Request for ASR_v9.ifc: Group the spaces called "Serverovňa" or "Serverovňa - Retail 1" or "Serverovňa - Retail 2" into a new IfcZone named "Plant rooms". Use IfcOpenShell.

First a look at what the model holds.

```python
import ifcopenshell

model = ifcopenshell.open("ASR_v9.ifc")
print(model.schema)
seen = {}
for space in model.by_type("IfcSpace"):
    seen[space.LongName] = seen.get(space.LongName, 0) + 1
for name, count in sorted(seen.items(), key=str):
    print(count, "x", name)
print("zones:", [z.Name for z in model.by_type("IfcZone")][:20])
```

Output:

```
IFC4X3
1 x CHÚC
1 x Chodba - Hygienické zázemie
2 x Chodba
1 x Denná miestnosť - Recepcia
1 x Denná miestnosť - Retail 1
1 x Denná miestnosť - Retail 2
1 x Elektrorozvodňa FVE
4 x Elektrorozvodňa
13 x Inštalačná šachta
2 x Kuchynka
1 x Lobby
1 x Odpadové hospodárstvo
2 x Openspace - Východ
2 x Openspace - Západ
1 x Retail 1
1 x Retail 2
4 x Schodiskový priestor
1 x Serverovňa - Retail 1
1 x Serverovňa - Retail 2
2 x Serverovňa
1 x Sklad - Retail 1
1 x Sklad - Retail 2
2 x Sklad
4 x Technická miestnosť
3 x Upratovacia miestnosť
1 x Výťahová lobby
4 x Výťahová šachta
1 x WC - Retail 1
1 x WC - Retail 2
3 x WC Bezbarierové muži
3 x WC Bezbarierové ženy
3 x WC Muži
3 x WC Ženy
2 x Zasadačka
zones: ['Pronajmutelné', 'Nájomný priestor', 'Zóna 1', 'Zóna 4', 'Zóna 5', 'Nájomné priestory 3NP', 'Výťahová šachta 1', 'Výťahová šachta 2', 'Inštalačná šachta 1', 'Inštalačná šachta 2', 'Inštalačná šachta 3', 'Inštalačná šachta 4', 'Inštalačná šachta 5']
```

```python
import ifcopenshell
import ifcopenshell.api.group
import ifcopenshell.api.root

model = ifcopenshell.open("ASR_v9.ifc")

names = {"Serverovňa", "Serverovňa - Retail 1", "Serverovňa - Retail 2"}
spaces = [s for s in model.by_type("IfcSpace") if s.LongName in names]

zone = ifcopenshell.api.root.create_entity(model, ifc_class="IfcZone", name="Plant rooms")
ifcopenshell.api.group.assign_group(model, products=spaces, group=zone)
print(len(spaces), "spaces in", zone.Name)

model.write("ASR_v9_updated.ifc")
```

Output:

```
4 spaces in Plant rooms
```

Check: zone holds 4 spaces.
